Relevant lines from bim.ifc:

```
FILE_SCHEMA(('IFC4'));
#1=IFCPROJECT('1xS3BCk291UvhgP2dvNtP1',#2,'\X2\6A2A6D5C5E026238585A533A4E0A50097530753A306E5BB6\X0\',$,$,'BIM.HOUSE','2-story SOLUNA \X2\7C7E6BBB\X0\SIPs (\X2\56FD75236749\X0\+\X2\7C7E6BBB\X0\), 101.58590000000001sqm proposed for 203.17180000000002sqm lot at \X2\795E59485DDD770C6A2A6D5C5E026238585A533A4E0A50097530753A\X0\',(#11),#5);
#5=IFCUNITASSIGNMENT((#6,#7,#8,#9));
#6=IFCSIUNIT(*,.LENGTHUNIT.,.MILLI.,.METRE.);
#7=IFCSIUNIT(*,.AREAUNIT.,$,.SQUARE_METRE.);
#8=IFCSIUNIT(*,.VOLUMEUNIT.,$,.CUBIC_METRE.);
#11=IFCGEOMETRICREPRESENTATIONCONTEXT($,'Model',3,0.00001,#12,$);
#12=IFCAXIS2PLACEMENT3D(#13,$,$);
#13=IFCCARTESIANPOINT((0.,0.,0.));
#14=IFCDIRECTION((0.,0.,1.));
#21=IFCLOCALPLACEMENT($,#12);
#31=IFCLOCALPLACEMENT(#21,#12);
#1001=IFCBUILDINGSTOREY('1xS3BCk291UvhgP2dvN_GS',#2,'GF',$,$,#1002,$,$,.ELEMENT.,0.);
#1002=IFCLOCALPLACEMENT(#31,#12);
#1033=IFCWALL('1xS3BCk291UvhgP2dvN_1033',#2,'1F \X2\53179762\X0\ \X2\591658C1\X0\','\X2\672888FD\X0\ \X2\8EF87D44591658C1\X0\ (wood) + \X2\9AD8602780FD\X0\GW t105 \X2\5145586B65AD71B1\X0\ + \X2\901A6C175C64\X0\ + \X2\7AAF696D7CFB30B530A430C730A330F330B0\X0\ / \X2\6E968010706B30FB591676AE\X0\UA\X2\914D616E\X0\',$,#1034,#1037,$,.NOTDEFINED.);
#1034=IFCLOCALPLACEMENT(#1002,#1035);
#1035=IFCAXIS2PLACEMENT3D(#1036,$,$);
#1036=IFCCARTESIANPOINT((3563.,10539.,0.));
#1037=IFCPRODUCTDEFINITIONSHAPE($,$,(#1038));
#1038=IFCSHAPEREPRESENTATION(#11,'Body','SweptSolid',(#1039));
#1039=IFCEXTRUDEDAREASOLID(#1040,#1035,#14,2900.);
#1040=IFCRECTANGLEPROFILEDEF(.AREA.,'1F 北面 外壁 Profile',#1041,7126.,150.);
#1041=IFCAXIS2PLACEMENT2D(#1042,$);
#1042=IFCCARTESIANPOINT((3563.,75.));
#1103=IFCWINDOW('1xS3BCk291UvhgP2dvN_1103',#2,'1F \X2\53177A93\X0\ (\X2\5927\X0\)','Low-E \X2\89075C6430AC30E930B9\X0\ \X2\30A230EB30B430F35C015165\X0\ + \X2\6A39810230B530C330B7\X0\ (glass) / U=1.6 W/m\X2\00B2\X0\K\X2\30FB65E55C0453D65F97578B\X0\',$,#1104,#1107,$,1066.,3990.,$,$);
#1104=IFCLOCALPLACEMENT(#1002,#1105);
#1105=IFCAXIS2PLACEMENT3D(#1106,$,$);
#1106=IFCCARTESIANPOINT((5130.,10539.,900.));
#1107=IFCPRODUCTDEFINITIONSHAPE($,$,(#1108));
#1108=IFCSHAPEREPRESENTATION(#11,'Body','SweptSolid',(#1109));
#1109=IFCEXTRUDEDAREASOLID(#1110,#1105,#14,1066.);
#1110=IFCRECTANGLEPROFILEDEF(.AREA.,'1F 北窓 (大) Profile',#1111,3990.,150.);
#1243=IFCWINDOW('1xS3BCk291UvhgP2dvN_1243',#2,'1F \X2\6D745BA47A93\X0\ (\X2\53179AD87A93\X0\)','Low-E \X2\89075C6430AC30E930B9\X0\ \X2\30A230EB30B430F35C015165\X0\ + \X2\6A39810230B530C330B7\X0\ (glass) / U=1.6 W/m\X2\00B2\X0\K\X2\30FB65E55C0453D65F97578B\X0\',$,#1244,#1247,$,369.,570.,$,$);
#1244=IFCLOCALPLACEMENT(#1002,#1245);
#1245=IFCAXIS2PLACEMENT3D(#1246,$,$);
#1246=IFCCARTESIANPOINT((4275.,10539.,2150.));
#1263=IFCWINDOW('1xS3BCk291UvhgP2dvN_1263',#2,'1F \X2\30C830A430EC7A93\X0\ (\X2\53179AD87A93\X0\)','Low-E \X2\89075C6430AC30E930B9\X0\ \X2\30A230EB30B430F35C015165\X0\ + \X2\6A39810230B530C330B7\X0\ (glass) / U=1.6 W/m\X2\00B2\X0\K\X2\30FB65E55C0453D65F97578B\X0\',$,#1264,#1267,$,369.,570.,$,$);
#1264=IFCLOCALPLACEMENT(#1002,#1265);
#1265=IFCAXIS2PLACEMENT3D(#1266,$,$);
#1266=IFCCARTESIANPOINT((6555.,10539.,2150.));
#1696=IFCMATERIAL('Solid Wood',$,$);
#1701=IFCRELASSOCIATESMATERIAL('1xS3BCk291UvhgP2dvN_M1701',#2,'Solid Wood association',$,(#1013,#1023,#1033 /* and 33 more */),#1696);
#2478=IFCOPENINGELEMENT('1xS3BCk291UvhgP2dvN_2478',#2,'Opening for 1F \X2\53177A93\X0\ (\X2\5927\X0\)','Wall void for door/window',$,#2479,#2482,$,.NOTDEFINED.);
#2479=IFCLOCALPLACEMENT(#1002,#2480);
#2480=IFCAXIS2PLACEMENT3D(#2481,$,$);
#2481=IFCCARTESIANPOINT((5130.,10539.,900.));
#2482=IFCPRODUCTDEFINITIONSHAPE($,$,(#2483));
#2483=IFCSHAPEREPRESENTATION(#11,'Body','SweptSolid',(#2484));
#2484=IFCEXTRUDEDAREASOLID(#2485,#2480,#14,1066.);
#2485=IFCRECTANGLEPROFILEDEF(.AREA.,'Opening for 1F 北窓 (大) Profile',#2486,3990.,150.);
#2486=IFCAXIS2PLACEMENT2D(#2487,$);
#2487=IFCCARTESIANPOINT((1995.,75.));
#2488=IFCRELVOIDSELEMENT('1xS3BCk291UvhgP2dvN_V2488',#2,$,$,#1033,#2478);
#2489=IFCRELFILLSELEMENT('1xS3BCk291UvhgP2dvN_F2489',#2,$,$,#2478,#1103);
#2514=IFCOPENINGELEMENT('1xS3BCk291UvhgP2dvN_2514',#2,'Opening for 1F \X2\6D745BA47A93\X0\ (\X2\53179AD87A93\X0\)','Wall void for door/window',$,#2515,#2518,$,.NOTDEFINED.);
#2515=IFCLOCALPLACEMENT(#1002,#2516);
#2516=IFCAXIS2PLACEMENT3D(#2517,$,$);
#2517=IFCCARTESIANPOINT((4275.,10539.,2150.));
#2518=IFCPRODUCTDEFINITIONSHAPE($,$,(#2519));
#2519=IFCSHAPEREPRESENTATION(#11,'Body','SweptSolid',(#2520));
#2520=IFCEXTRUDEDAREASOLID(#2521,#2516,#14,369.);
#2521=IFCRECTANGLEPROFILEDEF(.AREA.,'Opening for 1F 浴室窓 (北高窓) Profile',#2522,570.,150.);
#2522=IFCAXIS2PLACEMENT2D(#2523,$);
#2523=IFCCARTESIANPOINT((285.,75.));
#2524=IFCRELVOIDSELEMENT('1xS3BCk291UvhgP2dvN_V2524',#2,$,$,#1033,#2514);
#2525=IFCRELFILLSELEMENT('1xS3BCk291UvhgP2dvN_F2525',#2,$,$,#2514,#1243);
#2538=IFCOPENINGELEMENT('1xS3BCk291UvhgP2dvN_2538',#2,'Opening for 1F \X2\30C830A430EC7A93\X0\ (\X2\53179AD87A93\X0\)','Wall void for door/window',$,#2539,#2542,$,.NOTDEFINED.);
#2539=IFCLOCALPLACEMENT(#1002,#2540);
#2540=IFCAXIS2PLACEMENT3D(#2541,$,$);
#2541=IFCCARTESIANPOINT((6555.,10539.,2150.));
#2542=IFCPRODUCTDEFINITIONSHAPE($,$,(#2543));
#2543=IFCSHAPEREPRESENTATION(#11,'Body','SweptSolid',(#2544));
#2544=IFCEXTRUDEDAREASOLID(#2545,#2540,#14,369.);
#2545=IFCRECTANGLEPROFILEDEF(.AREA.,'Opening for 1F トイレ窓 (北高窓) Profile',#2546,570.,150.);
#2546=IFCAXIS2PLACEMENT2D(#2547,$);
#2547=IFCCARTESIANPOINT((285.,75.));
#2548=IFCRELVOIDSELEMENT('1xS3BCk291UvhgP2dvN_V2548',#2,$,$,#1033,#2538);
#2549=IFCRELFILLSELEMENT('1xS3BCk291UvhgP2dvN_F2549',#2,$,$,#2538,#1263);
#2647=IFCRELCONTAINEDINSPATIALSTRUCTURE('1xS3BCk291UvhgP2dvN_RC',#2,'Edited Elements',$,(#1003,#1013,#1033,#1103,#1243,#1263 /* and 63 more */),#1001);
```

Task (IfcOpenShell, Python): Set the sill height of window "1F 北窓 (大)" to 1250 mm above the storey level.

```python
import numpy as np
import ifcopenshell
import ifcopenshell.api.geometry
import ifcopenshell.geom
import ifcopenshell.util.element
import ifcopenshell.util.placement
import ifcopenshell.util.shape
import ifcopenshell.util.unit

model = ifcopenshell.open("bim.ifc")
unit_scale = ifcopenshell.util.unit.calculate_unit_scale(model)

window = model.by_id(1103)
opening = window.FillsVoids[0].RelatingOpeningElement
storey = ifcopenshell.util.element.get_container(window, ifc_class="IfcBuildingStorey")
level = ifcopenshell.util.placement.get_local_placement(storey.ObjectPlacement)[2, 3]

# The opening's origin need not be at the sill, so measure its lowest point.
shape = ifcopenshell.geom.create_shape(ifcopenshell.geom.settings(), opening)
bottom = ifcopenshell.util.shape.get_shape_bottom_elevation(shape, shape.geometry) / unit_scale
dz = level + 1.25 / unit_scale - bottom

shift = np.array([0.0, 0.0, dz])
# The window is not placed relative to its opening, so move both.
for product in (opening, window):
    matrix = ifcopenshell.util.placement.get_local_placement(product.ObjectPlacement)
    matrix[:3, 3] += shift
    ifcopenshell.api.geometry.edit_object_placement(model, product=product, matrix=matrix, is_si=False)

print(f"moved by {dz * unit_scale:+.3f} m")

model.write("bim_rev.ifc")
```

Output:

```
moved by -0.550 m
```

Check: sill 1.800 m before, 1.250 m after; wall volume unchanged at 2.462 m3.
